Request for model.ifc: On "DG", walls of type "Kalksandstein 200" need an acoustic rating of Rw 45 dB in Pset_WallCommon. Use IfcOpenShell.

First a look at what the model holds.

```python
import ifcopenshell
import ifcopenshell.util.element

model = ifcopenshell.open("model.ifc")
print(model.schema)
storey = next(s for s in model.by_type("IfcBuildingStorey") if s.Name == "DG")
walls = [e for e in ifcopenshell.util.element.get_decomposition(storey) if e.is_a("IfcWall")]
seen = {}
for e in walls:
    element_type = ifcopenshell.util.element.get_type(e)
    key = (element_type.Name if element_type != e and element_type else None, ifcopenshell.util.element.get_pset(e, "Pset_WallCommon", "AcousticRating"))
    seen[key] = seen.get(key, 0) + 1
for (name, value), count in sorted(seen.items(), key=str):
    print(count, "x", name, "|", value)
```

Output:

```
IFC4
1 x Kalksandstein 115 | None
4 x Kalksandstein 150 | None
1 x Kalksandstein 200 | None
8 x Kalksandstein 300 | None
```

```python
import ifcopenshell
import ifcopenshell.api.pset
import ifcopenshell.util.element

model = ifcopenshell.open("model.ifc")

storey = next(s for s in model.by_type("IfcBuildingStorey") if s.Name == "DG")
walls = [e for e in ifcopenshell.util.element.get_decomposition(storey) if e.is_a("IfcWall")]

count = 0
for e in walls:
    element_type = ifcopenshell.util.element.get_type(e)
    if element_type in (None, e) or element_type.Name != "Kalksandstein 200":
        continue
    # add_pset returns the element's existing set when there is one.
    pset = ifcopenshell.api.pset.add_pset(model, product=e, name="Pset_WallCommon")
    ifcopenshell.api.pset.edit_pset(model, pset=pset, properties={"AcousticRating": "Rw 45 dB"})
    count += 1

print(count, "walls updated")

model.write("model_rev.ifc")
```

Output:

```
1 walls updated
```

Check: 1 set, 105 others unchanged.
